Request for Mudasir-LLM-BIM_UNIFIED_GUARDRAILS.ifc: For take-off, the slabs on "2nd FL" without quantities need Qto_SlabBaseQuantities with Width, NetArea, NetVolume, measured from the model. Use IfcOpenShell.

First a look at what the model holds.

```python
import ifcopenshell
import ifcopenshell.util.element
import ifcopenshell.util.unit

model = ifcopenshell.open("Mudasir-LLM-BIM_UNIFIED_GUARDRAILS.ifc")
print(model.schema)
for unit_type in ("LENGTHUNIT", "AREAUNIT", "VOLUMEUNIT"):
    print(unit_type, ifcopenshell.util.unit.calculate_unit_scale(model, unit_type))
storey = next(s for s in model.by_type("IfcBuildingStorey") if s.Name == "2nd FL")
slabs = [e for e in ifcopenshell.util.element.get_decomposition(storey) if e.is_a("IfcSlab")]
for e in sorted(slabs, key=lambda e: e.id()):
    print(e.id(), e.is_a(), e.Name, list(ifcopenshell.util.element.get_psets(e, qtos_only=True)), sep=" | ")
```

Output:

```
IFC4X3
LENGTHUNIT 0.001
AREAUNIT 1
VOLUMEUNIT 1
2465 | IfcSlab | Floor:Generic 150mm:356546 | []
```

```python
import ifcopenshell
import ifcopenshell.api.pset
import ifcopenshell.geom
import ifcopenshell.util.element
import ifcopenshell.util.shape
import ifcopenshell.util.unit

model = ifcopenshell.open("Mudasir-LLM-BIM_UNIFIED_GUARDRAILS.ifc")
unit_scale = ifcopenshell.util.unit.calculate_unit_scale(model)
area_scale = ifcopenshell.util.unit.calculate_unit_scale(model, "AREAUNIT")
volume_scale = ifcopenshell.util.unit.calculate_unit_scale(model, "VOLUMEUNIT")
settings = ifcopenshell.geom.settings()

storey = next(s for s in model.by_type("IfcBuildingStorey") if s.Name == "2nd FL")
slabs = [e for e in ifcopenshell.util.element.get_decomposition(storey) if e.is_a("IfcSlab")]

for e in sorted(slabs, key=lambda e: e.id()):
    if ifcopenshell.util.element.get_psets(e, qtos_only=True, should_inherit=False):
        continue
    # Geometry comes back in metres, in the element's own axes.
    shape = ifcopenshell.geom.create_shape(settings, e)
    values = {
        "Width": ifcopenshell.util.shape.get_z(shape.geometry) / unit_scale,
        "NetArea": ifcopenshell.util.shape.get_footprint_area(shape.geometry) / area_scale,
        "NetVolume": ifcopenshell.util.shape.get_volume(shape.geometry) / volume_scale,
    }
    qto = ifcopenshell.api.pset.add_qto(model, product=e, name="Qto_SlabBaseQuantities")
    ifcopenshell.api.pset.edit_qto(model, qto=qto, properties=values)
    print(e.id(), {k: round(v, 3) for k, v in values.items()})

model.write("Mudasir-LLM-BIM_UNIFIED_GUARDRAILS_edited.ifc")
```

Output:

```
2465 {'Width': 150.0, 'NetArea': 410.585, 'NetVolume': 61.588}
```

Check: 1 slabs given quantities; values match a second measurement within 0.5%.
